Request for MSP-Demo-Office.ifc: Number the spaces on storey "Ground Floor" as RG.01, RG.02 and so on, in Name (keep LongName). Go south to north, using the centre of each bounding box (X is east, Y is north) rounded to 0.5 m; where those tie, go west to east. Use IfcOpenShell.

First a look at what the model holds.

```python
import ifcopenshell
import ifcopenshell.util.element
import ifcopenshell.util.placement

model = ifcopenshell.open("MSP-Demo-Office.ifc")
print(model.schema)
storey = next(s for s in model.by_type("IfcBuildingStorey") if s.Name == "Ground Floor")
spaces = [e for e in ifcopenshell.util.element.get_decomposition(storey) if e.is_a("IfcSpace")]
for e in sorted(spaces, key=lambda e: e.id()):
    origin = ifcopenshell.util.placement.get_local_placement(e.ObjectPlacement)[:3, 3]
    print(e.id(), e.Name, e.LongName, origin.round(2) + 0.0, sep=" | ")
```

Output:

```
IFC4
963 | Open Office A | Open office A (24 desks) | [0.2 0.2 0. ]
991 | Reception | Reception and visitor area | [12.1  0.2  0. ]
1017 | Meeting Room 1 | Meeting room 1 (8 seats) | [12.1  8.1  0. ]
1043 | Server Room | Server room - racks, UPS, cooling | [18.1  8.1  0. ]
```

```python
import ifcopenshell
import ifcopenshell.geom
import ifcopenshell.util.element
import ifcopenshell.util.shape

model = ifcopenshell.open("MSP-Demo-Office.ifc")
settings = ifcopenshell.geom.settings()
settings.set("use-world-coords", True)


def centre(element):
    shape = ifcopenshell.geom.create_shape(settings, element)
    return ifcopenshell.util.shape.get_bbox_centroid(shape.geometry)


storey = next(s for s in model.by_type("IfcBuildingStorey") if s.Name == "Ground Floor")
spaces = [e for e in ifcopenshell.util.element.get_decomposition(storey) if e.is_a("IfcSpace")]

# Insertion points can sit at a corner or the storey origin, so sort by the geometry (in metres).
centres = {e: centre(e) for e in spaces}
spaces.sort(key=lambda e: (round(centres[e][1] / 0.5), centres[e][0]))

for i, e in enumerate(spaces, start=1):
    number = f"RG.{i:02d}"
    e.Name = number
    print(e.id(), number)

model.write("MSP-Demo-Office_edited.ifc")
```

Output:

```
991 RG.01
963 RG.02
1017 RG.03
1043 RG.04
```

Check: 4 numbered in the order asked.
